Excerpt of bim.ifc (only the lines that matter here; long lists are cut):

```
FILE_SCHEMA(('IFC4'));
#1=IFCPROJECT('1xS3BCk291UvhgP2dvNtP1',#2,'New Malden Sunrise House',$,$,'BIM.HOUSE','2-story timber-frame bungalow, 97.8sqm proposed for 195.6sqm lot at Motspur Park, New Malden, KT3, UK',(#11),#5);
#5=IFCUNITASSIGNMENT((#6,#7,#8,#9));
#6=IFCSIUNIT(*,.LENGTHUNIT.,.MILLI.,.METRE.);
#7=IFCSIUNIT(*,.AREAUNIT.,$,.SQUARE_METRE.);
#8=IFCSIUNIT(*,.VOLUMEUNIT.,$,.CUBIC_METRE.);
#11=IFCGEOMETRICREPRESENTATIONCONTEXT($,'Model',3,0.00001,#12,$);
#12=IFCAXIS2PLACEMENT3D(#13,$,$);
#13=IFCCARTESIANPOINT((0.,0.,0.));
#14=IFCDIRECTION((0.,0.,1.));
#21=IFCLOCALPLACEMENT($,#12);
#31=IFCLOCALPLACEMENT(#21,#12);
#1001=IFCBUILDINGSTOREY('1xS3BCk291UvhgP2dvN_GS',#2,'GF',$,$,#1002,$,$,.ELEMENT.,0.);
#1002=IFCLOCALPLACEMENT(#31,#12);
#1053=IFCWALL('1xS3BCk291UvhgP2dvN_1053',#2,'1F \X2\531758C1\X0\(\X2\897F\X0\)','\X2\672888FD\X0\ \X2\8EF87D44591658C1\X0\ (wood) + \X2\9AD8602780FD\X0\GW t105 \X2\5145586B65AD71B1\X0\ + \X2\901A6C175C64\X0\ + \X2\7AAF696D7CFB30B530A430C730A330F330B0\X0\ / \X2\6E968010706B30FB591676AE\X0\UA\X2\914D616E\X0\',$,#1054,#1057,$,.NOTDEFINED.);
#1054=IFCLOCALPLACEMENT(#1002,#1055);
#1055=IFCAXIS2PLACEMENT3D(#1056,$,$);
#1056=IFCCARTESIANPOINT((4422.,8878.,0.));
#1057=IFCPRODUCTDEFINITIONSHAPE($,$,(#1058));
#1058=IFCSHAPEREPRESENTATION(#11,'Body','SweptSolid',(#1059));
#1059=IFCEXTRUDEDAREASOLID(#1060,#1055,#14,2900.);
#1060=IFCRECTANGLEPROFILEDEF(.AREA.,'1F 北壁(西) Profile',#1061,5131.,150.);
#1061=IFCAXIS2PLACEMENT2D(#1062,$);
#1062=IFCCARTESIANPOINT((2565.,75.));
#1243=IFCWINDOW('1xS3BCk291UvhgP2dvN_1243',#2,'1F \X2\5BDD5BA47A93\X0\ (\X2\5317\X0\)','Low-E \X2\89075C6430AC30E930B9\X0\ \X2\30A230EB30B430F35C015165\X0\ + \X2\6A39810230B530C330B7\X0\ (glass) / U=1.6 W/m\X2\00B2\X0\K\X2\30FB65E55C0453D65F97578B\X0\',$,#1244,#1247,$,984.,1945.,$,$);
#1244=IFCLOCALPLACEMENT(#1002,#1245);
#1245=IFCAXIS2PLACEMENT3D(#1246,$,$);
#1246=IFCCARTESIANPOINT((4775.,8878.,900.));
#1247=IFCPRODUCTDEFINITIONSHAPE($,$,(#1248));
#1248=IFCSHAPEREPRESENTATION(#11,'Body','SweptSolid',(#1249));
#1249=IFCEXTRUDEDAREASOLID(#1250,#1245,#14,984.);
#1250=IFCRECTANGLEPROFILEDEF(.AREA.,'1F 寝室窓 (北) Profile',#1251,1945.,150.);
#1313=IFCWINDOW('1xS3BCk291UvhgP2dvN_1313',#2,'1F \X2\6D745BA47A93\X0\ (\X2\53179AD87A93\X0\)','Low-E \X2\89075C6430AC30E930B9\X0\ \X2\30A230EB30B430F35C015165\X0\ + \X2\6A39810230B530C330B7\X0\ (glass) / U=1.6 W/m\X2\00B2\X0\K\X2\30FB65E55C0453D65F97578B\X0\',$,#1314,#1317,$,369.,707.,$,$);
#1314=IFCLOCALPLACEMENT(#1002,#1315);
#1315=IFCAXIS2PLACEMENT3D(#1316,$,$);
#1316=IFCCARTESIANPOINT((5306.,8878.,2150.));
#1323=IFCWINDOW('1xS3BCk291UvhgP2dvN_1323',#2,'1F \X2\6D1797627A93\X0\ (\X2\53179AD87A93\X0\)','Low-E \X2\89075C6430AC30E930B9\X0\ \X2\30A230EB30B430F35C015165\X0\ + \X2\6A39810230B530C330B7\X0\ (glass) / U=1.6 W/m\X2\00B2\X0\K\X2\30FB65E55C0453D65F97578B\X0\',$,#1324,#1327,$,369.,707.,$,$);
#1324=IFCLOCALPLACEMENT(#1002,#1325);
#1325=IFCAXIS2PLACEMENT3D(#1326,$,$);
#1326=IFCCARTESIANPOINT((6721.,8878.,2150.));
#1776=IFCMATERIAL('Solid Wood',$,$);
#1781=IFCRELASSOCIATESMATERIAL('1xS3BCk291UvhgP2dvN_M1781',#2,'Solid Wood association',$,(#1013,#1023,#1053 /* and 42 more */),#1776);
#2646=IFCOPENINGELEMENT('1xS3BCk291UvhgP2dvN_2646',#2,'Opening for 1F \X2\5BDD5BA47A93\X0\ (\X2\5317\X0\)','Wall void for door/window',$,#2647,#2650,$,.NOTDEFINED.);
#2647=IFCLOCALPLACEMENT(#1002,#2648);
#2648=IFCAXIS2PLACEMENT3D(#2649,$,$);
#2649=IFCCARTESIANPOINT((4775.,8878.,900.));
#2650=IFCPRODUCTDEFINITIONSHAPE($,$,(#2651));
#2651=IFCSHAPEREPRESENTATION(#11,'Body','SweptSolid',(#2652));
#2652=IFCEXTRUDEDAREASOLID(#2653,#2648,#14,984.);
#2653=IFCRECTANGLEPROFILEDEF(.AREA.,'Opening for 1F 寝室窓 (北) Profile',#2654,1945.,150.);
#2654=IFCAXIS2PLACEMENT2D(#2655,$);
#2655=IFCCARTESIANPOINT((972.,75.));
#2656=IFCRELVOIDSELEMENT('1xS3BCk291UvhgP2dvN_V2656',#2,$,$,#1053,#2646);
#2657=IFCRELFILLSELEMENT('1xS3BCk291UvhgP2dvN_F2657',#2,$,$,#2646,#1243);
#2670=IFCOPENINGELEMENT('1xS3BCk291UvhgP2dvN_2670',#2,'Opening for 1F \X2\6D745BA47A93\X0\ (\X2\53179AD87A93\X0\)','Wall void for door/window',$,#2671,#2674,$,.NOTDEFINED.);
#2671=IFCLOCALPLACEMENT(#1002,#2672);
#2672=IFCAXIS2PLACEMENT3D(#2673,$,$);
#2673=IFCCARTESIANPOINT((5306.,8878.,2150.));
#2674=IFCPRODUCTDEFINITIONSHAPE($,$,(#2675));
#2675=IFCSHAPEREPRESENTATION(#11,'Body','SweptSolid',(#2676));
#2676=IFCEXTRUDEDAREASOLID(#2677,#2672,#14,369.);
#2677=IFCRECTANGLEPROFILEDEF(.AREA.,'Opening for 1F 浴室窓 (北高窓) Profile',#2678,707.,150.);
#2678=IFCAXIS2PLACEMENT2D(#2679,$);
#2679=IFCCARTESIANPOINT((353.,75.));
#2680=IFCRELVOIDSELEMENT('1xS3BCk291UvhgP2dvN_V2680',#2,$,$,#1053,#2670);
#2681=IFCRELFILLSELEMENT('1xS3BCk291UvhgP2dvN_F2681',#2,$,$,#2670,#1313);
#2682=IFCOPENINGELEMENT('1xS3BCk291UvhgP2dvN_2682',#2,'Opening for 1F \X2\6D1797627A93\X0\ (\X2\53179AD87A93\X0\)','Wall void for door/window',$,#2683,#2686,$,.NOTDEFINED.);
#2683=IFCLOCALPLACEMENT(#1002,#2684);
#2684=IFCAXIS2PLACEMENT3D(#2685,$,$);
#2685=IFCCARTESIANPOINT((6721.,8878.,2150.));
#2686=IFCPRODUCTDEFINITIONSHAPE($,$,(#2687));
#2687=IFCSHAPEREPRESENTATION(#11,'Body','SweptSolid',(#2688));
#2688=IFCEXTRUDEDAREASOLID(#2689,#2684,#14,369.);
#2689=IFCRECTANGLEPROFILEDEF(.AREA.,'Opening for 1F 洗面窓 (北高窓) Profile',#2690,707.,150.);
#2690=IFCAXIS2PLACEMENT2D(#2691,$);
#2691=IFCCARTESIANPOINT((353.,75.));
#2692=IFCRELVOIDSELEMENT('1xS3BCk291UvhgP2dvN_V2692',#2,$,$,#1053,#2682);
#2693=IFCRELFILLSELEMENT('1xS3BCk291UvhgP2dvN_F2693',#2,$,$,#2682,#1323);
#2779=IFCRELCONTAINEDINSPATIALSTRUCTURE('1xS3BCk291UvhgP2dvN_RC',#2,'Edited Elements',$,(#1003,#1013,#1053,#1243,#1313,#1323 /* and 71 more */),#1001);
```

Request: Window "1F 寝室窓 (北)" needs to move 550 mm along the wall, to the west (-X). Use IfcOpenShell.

```python
import ifcopenshell
import ifcopenshell.api.geometry
import ifcopenshell.util.placement
import ifcopenshell.util.unit

model = ifcopenshell.open("bim.ifc")
unit_scale = ifcopenshell.util.unit.calculate_unit_scale(model)

window = model.by_guid("1xS3BCk291UvhgP2dvN_1243")
opening = window.FillsVoids[0].RelatingOpeningElement
wall = opening.VoidsElements[0].RelatingBuildingElement

wall_matrix = ifcopenshell.util.placement.get_local_placement(wall.ObjectPlacement)
shift = wall_matrix[:3, 0] * -0.55 / unit_scale
before = ifcopenshell.util.placement.get_local_placement(window.ObjectPlacement)[:3, 3].copy()

# The window is not placed relative to its opening, so move both.
for product in (opening, window):
    matrix = ifcopenshell.util.placement.get_local_placement(product.ObjectPlacement)
    matrix[:3, 3] += shift
    ifcopenshell.api.geometry.edit_object_placement(model, product=product, matrix=matrix, is_si=False)

after = ifcopenshell.util.placement.get_local_placement(window.ObjectPlacement)[:3, 3]
print("window moved by", (after - before).round(3) + 0.0)

model.write("bim_rev.ifc")
```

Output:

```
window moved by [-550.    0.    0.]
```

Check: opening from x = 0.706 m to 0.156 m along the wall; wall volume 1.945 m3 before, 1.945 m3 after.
